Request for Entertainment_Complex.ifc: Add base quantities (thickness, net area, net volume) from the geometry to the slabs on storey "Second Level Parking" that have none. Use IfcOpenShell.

First a look at what the model holds.

```python
import ifcopenshell
import ifcopenshell.util.element
import ifcopenshell.util.unit

model = ifcopenshell.open("Entertainment_Complex.ifc")
print(model.schema)
for unit_type in ("LENGTHUNIT", "AREAUNIT", "VOLUMEUNIT"):
    print(unit_type, ifcopenshell.util.unit.calculate_unit_scale(model, unit_type))
storey = next(s for s in model.by_type("IfcBuildingStorey") if s.Name == "Second Level Parking")
slabs = [e for e in ifcopenshell.util.element.get_decomposition(storey) if e.is_a("IfcSlab")]
for e in sorted(slabs, key=lambda e: e.id()):
    print(e.id(), e.is_a(), e.Name, list(ifcopenshell.util.element.get_psets(e, qtos_only=True)), sep=" | ")
```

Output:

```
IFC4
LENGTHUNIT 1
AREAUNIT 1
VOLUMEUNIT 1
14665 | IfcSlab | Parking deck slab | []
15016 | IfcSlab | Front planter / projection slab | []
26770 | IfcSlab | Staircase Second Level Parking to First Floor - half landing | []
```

```python
import ifcopenshell
import ifcopenshell.api.pset
import ifcopenshell.geom
import ifcopenshell.util.element
import ifcopenshell.util.shape
import ifcopenshell.util.unit

model = ifcopenshell.open("Entertainment_Complex.ifc")
unit_scale = ifcopenshell.util.unit.calculate_unit_scale(model)
area_scale = ifcopenshell.util.unit.calculate_unit_scale(model, "AREAUNIT")
volume_scale = ifcopenshell.util.unit.calculate_unit_scale(model, "VOLUMEUNIT")
settings = ifcopenshell.geom.settings()

storey = next(s for s in model.by_type("IfcBuildingStorey") if s.Name == "Second Level Parking")
slabs = [e for e in ifcopenshell.util.element.get_decomposition(storey) if e.is_a("IfcSlab")]

for e in sorted(slabs, key=lambda e: e.id()):
    if ifcopenshell.util.element.get_psets(e, qtos_only=True, should_inherit=False):
        continue
    # Geometry comes back in metres, in the element's own axes.
    shape = ifcopenshell.geom.create_shape(settings, e)
    values = {
        "Width": ifcopenshell.util.shape.get_z(shape.geometry) / unit_scale,
        "NetArea": ifcopenshell.util.shape.get_footprint_area(shape.geometry) / area_scale,
        "NetVolume": ifcopenshell.util.shape.get_volume(shape.geometry) / volume_scale,
    }
    qto = ifcopenshell.api.pset.add_qto(model, product=e, name="Qto_SlabBaseQuantities")
    ifcopenshell.api.pset.edit_qto(model, qto=qto, properties=values)
    print(e.id(), {k: round(v, 3) for k, v in values.items()})

model.write("Entertainment_Complex_rev.ifc")
```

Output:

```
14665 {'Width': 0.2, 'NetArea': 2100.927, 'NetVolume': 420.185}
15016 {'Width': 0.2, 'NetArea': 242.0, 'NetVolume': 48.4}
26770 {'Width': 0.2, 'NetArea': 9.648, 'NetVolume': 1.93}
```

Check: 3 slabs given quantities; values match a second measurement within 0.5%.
